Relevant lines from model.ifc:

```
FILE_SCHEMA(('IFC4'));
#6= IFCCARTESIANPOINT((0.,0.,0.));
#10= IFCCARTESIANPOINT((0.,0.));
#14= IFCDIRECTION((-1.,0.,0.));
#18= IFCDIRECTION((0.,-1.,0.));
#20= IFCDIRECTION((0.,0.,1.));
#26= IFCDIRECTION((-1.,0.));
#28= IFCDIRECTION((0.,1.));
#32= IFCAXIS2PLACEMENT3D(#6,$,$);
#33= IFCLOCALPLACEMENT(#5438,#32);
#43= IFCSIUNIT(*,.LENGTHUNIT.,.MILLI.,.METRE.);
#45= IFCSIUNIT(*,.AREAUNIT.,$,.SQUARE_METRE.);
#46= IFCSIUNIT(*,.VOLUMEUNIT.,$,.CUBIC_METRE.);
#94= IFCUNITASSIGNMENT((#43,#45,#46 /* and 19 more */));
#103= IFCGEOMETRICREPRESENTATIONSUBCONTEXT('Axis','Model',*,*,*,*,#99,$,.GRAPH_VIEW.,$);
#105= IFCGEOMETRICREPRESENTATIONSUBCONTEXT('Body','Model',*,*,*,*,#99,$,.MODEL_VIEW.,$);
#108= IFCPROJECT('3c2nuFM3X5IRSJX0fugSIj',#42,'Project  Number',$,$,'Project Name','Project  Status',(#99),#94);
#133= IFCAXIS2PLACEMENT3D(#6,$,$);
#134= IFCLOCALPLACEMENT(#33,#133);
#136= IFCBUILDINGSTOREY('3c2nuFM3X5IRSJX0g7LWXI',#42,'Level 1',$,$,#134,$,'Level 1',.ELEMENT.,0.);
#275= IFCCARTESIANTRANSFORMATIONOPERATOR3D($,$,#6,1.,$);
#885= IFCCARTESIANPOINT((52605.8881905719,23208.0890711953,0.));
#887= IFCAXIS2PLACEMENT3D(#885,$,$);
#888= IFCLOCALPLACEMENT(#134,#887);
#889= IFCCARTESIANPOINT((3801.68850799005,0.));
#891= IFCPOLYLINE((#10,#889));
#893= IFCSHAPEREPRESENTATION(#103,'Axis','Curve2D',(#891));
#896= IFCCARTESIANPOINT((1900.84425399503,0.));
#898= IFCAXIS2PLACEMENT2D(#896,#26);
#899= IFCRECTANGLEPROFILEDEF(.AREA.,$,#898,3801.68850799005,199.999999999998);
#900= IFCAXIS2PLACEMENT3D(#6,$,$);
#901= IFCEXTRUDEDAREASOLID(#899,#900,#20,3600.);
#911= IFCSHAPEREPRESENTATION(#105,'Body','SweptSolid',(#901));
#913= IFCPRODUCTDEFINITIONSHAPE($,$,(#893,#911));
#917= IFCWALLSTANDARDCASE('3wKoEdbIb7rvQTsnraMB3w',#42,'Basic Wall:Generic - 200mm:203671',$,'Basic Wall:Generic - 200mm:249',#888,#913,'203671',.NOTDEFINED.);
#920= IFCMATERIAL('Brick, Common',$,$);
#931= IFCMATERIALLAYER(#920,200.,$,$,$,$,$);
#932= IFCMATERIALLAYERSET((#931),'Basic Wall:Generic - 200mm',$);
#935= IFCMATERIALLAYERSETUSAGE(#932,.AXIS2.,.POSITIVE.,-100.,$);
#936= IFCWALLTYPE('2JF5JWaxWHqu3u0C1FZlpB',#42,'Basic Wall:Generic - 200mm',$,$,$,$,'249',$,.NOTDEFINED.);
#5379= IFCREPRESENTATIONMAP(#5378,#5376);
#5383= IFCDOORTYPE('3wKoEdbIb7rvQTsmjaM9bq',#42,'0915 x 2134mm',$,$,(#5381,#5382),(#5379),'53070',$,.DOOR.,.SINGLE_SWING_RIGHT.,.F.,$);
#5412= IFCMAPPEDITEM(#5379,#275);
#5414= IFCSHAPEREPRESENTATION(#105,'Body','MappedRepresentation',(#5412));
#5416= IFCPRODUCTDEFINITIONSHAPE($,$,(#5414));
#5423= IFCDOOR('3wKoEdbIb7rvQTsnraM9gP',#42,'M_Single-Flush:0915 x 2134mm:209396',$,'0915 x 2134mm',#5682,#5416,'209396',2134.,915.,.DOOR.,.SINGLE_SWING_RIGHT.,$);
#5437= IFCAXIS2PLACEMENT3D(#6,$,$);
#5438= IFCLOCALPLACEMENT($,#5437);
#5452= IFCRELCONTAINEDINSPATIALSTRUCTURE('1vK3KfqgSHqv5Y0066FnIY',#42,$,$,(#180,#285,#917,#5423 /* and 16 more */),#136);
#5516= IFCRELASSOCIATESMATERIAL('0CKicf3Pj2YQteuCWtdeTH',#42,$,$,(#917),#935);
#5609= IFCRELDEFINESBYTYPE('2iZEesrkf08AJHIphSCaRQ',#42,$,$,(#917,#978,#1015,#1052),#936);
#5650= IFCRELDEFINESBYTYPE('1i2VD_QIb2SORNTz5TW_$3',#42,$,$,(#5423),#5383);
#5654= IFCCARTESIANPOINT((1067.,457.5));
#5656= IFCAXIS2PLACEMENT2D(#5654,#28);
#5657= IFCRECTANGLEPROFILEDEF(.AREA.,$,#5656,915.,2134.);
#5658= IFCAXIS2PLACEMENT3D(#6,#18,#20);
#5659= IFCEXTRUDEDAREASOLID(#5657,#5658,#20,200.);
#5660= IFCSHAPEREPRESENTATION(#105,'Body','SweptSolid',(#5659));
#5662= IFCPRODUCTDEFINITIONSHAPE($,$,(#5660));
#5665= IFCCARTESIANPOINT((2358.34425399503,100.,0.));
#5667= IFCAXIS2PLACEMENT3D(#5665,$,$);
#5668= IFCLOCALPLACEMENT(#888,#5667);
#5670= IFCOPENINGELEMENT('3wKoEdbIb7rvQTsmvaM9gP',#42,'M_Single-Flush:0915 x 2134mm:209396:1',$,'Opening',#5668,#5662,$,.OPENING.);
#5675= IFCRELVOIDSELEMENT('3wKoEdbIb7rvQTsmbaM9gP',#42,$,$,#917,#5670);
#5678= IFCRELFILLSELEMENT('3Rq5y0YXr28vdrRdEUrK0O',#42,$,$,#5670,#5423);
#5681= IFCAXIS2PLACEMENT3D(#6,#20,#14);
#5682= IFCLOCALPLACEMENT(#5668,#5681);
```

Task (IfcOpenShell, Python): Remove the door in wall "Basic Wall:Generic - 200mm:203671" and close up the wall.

```python
import ifcopenshell
import ifcopenshell.api.feature
import ifcopenshell.api.root
import ifcopenshell.geom
import ifcopenshell.util.shape

model = ifcopenshell.open("model.ifc")
settings = ifcopenshell.geom.settings()


def volume(element):
    """Net volume in cubic metres, openings subtracted."""
    shape = ifcopenshell.geom.create_shape(settings, element)
    return ifcopenshell.util.shape.get_volume(shape.geometry)


door = model.by_id(5423)
opening = door.FillsVoids[0].RelatingOpeningElement
wall = opening.VoidsElements[0].RelatingBuildingElement
before = volume(wall)

ifcopenshell.api.root.remove_product(model, product=door)
ifcopenshell.api.feature.remove_feature(model, feature=opening)

after = volume(wall)

print(f"wall volume {before:.3f} -> {after:.3f} m3")

model.write("model_rev.ifc")
```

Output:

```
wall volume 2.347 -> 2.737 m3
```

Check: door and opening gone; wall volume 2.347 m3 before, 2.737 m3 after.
